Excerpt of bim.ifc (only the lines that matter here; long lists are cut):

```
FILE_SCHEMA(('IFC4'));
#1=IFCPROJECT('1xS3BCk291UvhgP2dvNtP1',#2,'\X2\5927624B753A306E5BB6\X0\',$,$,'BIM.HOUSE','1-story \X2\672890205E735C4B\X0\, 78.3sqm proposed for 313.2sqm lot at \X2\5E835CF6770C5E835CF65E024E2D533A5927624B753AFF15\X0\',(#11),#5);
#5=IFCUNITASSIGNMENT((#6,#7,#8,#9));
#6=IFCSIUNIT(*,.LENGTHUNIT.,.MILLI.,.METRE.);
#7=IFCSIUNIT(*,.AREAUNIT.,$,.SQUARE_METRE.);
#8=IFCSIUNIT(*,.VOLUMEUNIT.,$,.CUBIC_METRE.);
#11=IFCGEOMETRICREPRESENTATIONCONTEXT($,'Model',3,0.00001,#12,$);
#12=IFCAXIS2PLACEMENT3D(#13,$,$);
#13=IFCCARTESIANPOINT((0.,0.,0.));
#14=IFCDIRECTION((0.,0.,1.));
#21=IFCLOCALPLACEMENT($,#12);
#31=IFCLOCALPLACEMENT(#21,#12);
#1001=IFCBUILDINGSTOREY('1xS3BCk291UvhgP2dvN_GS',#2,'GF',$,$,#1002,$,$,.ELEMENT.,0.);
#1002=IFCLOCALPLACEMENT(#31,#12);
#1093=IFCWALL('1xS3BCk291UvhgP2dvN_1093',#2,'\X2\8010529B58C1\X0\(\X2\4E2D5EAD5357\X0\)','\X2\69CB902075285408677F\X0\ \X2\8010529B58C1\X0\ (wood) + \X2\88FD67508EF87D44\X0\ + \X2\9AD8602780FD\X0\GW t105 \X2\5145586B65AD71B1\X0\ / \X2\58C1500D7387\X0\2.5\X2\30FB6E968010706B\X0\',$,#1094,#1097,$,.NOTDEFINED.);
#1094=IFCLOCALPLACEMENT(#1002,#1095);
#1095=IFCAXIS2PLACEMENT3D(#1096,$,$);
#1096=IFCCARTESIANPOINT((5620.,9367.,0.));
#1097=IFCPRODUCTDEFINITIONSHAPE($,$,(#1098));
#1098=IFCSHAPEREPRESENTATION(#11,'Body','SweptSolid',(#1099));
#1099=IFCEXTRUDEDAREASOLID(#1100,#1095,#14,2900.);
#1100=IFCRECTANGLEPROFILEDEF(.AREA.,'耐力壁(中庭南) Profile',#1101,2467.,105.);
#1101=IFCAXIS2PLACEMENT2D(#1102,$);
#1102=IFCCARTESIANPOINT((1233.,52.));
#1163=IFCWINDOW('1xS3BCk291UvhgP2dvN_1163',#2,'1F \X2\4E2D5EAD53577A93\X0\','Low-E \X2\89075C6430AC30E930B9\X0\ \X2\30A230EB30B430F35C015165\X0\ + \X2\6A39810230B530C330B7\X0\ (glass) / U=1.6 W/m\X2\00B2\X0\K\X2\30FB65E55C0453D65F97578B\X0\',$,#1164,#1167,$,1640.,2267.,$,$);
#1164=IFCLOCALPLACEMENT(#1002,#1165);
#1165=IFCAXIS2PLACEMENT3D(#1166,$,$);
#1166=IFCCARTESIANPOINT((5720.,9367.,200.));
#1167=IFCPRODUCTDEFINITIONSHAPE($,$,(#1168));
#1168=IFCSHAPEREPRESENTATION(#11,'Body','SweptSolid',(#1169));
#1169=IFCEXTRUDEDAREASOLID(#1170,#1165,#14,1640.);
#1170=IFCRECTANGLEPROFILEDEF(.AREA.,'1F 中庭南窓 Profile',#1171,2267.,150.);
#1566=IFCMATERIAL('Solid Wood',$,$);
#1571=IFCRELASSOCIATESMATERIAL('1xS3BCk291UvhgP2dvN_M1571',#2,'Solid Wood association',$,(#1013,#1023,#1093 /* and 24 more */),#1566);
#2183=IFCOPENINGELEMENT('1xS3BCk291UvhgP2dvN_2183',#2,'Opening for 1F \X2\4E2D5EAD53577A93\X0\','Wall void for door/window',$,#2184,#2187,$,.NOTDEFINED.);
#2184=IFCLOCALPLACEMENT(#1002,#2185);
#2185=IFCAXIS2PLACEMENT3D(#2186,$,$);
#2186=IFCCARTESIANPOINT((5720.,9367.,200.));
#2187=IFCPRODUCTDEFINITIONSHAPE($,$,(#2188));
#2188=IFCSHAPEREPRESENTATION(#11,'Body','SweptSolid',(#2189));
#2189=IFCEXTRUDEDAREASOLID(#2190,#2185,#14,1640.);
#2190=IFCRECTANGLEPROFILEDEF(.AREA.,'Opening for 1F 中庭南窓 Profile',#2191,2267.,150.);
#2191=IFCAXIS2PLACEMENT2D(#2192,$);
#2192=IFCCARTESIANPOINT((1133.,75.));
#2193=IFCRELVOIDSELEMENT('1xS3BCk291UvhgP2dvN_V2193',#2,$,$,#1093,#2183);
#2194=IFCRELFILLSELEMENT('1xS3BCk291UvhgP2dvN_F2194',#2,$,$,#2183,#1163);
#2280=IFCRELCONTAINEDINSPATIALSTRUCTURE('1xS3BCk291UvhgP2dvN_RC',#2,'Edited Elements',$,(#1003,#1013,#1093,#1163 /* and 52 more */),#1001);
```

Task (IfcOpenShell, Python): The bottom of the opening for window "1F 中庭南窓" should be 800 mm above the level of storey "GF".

```python
import numpy as np
import ifcopenshell
import ifcopenshell.api.geometry
import ifcopenshell.geom
import ifcopenshell.util.element
import ifcopenshell.util.placement
import ifcopenshell.util.shape
import ifcopenshell.util.unit

model = ifcopenshell.open("bim.ifc")
unit_scale = ifcopenshell.util.unit.calculate_unit_scale(model)

window = model.by_id(1163)
opening = window.FillsVoids[0].RelatingOpeningElement
storey = ifcopenshell.util.element.get_container(window, ifc_class="IfcBuildingStorey")
level = ifcopenshell.util.placement.get_local_placement(storey.ObjectPlacement)[2, 3]

# The opening's origin need not be at the sill, so measure its lowest point.
shape = ifcopenshell.geom.create_shape(ifcopenshell.geom.settings(), opening)
bottom = ifcopenshell.util.shape.get_shape_bottom_elevation(shape, shape.geometry) / unit_scale
dz = level + 0.8 / unit_scale - bottom

shift = np.array([0.0, 0.0, dz])
# The window is not placed relative to its opening, so move both.
for product in (opening, window):
    matrix = ifcopenshell.util.placement.get_local_placement(product.ObjectPlacement)
    matrix[:3, 3] += shift
    ifcopenshell.api.geometry.edit_object_placement(model, product=product, matrix=matrix, is_si=False)

print(f"moved by {dz * unit_scale:+.3f} m")

model.write("bim_edited.ifc")
```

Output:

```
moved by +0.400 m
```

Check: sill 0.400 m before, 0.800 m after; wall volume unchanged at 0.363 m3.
